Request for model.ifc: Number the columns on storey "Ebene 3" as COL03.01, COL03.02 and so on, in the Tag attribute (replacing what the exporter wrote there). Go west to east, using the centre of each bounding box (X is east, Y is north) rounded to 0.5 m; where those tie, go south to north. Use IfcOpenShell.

First a look at what the model holds.

```python
import ifcopenshell
import ifcopenshell.util.element
import ifcopenshell.util.placement

model = ifcopenshell.open("model.ifc")
print(model.schema)
storey = next(s for s in model.by_type("IfcBuildingStorey") if s.Name == "Ebene 3")
columns = [e for e in ifcopenshell.util.element.get_decomposition(storey) if e.is_a("IfcColumn")]
for e in sorted(columns, key=lambda e: e.id()):
    origin = ifcopenshell.util.placement.get_local_placement(e.ObjectPlacement)[:3, 3]
    print(e.id(), e.Tag, e.Name, origin.round(2) + 0.0, sep=" | ")
```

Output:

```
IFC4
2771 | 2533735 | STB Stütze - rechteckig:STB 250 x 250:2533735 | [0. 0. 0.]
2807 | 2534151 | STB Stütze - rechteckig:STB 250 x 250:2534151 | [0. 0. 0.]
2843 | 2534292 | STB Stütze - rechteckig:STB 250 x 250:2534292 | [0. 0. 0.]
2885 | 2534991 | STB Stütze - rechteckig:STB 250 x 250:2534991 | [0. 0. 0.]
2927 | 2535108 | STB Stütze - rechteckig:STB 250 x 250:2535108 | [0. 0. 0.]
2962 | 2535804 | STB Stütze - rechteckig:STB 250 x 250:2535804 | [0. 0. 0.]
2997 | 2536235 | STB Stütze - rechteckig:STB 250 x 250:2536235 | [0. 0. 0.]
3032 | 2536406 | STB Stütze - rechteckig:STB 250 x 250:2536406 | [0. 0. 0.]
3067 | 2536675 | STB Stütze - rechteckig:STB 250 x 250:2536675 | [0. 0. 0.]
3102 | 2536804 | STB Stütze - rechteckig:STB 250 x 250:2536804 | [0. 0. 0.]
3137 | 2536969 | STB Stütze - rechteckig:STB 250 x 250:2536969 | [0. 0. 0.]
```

```python
import ifcopenshell
import ifcopenshell.geom
import ifcopenshell.util.element
import ifcopenshell.util.shape

model = ifcopenshell.open("model.ifc")
settings = ifcopenshell.geom.settings()
settings.set("use-world-coords", True)


def centre(element):
    shape = ifcopenshell.geom.create_shape(settings, element)
    return ifcopenshell.util.shape.get_bbox_centroid(shape.geometry)


storey = next(s for s in model.by_type("IfcBuildingStorey") if s.Name == "Ebene 3")
columns = [e for e in ifcopenshell.util.element.get_decomposition(storey) if e.is_a("IfcColumn")]

# Insertion points can sit at a corner or the storey origin, so sort by the geometry (in metres).
centres = {e: centre(e) for e in columns}
columns.sort(key=lambda e: (round(centres[e][0] / 0.5), centres[e][1]))

for i, e in enumerate(columns, start=1):
    number = f"COL03.{i:02d}"
    e.Tag = number
    print(e.id(), number)

model.write("model-out.ifc")
```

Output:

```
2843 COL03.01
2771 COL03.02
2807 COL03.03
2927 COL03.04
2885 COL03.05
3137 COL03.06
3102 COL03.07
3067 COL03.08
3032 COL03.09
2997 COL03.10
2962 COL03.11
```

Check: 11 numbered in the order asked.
